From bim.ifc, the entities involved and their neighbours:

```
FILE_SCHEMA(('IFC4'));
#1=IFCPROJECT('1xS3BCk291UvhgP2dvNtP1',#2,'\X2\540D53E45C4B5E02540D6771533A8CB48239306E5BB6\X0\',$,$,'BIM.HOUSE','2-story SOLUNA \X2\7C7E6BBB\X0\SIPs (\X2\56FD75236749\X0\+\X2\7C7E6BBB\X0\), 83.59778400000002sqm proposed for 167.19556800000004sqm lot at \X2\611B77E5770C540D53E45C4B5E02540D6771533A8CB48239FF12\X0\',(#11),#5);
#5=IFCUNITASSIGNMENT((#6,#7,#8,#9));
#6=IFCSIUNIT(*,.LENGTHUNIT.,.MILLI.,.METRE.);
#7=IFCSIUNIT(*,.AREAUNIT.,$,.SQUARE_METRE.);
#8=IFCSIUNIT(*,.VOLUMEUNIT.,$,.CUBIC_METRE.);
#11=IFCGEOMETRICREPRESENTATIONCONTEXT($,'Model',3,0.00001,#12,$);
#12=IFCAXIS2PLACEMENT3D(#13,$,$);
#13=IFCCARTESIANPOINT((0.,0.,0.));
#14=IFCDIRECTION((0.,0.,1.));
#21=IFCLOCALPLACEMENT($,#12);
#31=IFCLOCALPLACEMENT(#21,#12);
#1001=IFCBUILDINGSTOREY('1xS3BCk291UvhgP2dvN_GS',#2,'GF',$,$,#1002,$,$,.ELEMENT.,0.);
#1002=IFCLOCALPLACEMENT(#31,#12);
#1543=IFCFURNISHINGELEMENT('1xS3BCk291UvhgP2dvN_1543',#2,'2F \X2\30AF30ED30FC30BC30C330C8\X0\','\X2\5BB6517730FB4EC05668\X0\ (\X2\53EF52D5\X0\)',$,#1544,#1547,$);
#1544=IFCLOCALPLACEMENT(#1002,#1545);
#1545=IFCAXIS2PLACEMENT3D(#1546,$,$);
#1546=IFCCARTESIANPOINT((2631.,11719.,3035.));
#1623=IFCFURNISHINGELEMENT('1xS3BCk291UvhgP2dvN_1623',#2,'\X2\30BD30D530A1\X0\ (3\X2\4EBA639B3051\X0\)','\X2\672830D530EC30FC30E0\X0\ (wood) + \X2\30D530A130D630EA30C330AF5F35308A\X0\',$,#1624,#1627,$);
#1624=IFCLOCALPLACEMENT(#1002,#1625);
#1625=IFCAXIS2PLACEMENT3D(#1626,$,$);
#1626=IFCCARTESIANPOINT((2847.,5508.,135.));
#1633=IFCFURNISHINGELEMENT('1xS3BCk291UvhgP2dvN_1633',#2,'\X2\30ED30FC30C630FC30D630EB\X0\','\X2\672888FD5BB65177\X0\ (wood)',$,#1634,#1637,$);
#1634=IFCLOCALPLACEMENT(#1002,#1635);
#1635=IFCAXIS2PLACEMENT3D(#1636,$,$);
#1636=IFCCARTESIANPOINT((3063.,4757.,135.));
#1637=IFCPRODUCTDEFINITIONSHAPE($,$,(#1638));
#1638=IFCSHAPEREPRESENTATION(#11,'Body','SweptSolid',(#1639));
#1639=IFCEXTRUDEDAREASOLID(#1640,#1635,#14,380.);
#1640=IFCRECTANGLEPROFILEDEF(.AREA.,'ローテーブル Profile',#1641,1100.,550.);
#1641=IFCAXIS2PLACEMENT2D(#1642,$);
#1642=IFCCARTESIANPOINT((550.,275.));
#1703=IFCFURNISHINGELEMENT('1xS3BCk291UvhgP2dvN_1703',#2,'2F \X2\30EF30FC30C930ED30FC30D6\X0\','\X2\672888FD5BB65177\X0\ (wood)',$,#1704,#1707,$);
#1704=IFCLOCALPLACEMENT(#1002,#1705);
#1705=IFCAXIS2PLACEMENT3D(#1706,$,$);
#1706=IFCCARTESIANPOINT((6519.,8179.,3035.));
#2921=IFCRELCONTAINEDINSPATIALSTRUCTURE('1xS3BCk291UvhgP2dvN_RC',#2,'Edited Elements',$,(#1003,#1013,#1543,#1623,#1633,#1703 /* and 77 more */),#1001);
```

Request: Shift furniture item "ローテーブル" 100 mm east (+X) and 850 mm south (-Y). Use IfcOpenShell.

```python
import ifcopenshell
import ifcopenshell.api.geometry
import ifcopenshell.util.placement
import ifcopenshell.util.unit

model = ifcopenshell.open("bim.ifc")
unit_scale = ifcopenshell.util.unit.calculate_unit_scale(model)

item = model.by_id(1633)
matrix = ifcopenshell.util.placement.get_local_placement(item.ObjectPlacement)
matrix[0, 3] += 0.1 / unit_scale
matrix[1, 3] -= 0.85 / unit_scale
ifcopenshell.api.geometry.edit_object_placement(model, product=item, matrix=matrix, is_si=False)

print(ifcopenshell.util.placement.get_local_placement(item.ObjectPlacement).round(3) + 0.0)

model.write("bim_v2.ifc")
```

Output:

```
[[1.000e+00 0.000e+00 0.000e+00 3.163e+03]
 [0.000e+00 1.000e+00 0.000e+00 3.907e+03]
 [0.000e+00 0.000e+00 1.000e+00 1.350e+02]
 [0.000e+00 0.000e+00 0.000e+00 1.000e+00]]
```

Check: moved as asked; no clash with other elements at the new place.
